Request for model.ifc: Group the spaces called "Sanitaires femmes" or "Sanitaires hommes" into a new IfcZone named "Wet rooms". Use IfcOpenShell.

First a look at what the model holds.

```python
import ifcopenshell

model = ifcopenshell.open("model.ifc")
print(model.schema)
seen = {}
for space in model.by_type("IfcSpace"):
    seen[space.LongName] = seen.get(space.LongName, 0) + 1
for name, count in sorted(seen.items(), key=str):
    print(count, "x", name)
print("zones:", [z.Name for z in model.by_type("IfcZone")][:20])
```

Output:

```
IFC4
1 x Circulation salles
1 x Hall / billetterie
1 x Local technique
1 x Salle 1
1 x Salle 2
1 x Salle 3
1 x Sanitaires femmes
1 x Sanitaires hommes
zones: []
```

```python
import ifcopenshell
import ifcopenshell.api.group
import ifcopenshell.api.root

model = ifcopenshell.open("model.ifc")

names = {"Sanitaires femmes", "Sanitaires hommes"}
spaces = [s for s in model.by_type("IfcSpace") if s.LongName in names]

zone = ifcopenshell.api.root.create_entity(model, ifc_class="IfcZone", name="Wet rooms")
ifcopenshell.api.group.assign_group(model, products=spaces, group=zone)
print(len(spaces), "spaces in", zone.Name)

model.write("model_v2.ifc")
```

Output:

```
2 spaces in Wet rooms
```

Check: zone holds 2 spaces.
